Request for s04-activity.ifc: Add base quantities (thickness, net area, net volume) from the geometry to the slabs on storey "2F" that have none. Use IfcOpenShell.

First a look at what the model holds.

```python
import ifcopenshell
import ifcopenshell.util.element
import ifcopenshell.util.unit

model = ifcopenshell.open("s04-activity.ifc")
print(model.schema)
for unit_type in ("LENGTHUNIT", "AREAUNIT", "VOLUMEUNIT"):
    print(unit_type, ifcopenshell.util.unit.calculate_unit_scale(model, unit_type))
storey = next(s for s in model.by_type("IfcBuildingStorey") if s.Name == "2F")
slabs = [e for e in ifcopenshell.util.element.get_decomposition(storey) if e.is_a("IfcSlab")]
for e in sorted(slabs, key=lambda e: e.id()):
    print(e.id(), e.is_a(), e.Name, list(ifcopenshell.util.element.get_psets(e, qtos_only=True)), sep=" | ")
```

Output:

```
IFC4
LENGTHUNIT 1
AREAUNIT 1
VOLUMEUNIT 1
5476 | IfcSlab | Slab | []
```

```python
import ifcopenshell
import ifcopenshell.api.pset
import ifcopenshell.geom
import ifcopenshell.util.element
import ifcopenshell.util.shape
import ifcopenshell.util.unit

model = ifcopenshell.open("s04-activity.ifc")
unit_scale = ifcopenshell.util.unit.calculate_unit_scale(model)
area_scale = ifcopenshell.util.unit.calculate_unit_scale(model, "AREAUNIT")
volume_scale = ifcopenshell.util.unit.calculate_unit_scale(model, "VOLUMEUNIT")
settings = ifcopenshell.geom.settings()

storey = next(s for s in model.by_type("IfcBuildingStorey") if s.Name == "2F")
slabs = [e for e in ifcopenshell.util.element.get_decomposition(storey) if e.is_a("IfcSlab")]

for e in sorted(slabs, key=lambda e: e.id()):
    if ifcopenshell.util.element.get_psets(e, qtos_only=True, should_inherit=False):
        continue
    # Geometry comes back in metres, in the element's own axes.
    shape = ifcopenshell.geom.create_shape(settings, e)
    values = {
        "Width": ifcopenshell.util.shape.get_z(shape.geometry) / unit_scale,
        "NetArea": ifcopenshell.util.shape.get_footprint_area(shape.geometry) / area_scale,
        "NetVolume": ifcopenshell.util.shape.get_volume(shape.geometry) / volume_scale,
    }
    qto = ifcopenshell.api.pset.add_qto(model, product=e, name="Qto_SlabBaseQuantities")
    ifcopenshell.api.pset.edit_qto(model, qto=qto, properties=values)
    print(e.id(), {k: round(v, 3) for k, v in values.items()})

model.write("s04-activity_edited.ifc")
```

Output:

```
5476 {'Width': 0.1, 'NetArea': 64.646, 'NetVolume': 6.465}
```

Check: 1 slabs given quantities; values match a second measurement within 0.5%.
